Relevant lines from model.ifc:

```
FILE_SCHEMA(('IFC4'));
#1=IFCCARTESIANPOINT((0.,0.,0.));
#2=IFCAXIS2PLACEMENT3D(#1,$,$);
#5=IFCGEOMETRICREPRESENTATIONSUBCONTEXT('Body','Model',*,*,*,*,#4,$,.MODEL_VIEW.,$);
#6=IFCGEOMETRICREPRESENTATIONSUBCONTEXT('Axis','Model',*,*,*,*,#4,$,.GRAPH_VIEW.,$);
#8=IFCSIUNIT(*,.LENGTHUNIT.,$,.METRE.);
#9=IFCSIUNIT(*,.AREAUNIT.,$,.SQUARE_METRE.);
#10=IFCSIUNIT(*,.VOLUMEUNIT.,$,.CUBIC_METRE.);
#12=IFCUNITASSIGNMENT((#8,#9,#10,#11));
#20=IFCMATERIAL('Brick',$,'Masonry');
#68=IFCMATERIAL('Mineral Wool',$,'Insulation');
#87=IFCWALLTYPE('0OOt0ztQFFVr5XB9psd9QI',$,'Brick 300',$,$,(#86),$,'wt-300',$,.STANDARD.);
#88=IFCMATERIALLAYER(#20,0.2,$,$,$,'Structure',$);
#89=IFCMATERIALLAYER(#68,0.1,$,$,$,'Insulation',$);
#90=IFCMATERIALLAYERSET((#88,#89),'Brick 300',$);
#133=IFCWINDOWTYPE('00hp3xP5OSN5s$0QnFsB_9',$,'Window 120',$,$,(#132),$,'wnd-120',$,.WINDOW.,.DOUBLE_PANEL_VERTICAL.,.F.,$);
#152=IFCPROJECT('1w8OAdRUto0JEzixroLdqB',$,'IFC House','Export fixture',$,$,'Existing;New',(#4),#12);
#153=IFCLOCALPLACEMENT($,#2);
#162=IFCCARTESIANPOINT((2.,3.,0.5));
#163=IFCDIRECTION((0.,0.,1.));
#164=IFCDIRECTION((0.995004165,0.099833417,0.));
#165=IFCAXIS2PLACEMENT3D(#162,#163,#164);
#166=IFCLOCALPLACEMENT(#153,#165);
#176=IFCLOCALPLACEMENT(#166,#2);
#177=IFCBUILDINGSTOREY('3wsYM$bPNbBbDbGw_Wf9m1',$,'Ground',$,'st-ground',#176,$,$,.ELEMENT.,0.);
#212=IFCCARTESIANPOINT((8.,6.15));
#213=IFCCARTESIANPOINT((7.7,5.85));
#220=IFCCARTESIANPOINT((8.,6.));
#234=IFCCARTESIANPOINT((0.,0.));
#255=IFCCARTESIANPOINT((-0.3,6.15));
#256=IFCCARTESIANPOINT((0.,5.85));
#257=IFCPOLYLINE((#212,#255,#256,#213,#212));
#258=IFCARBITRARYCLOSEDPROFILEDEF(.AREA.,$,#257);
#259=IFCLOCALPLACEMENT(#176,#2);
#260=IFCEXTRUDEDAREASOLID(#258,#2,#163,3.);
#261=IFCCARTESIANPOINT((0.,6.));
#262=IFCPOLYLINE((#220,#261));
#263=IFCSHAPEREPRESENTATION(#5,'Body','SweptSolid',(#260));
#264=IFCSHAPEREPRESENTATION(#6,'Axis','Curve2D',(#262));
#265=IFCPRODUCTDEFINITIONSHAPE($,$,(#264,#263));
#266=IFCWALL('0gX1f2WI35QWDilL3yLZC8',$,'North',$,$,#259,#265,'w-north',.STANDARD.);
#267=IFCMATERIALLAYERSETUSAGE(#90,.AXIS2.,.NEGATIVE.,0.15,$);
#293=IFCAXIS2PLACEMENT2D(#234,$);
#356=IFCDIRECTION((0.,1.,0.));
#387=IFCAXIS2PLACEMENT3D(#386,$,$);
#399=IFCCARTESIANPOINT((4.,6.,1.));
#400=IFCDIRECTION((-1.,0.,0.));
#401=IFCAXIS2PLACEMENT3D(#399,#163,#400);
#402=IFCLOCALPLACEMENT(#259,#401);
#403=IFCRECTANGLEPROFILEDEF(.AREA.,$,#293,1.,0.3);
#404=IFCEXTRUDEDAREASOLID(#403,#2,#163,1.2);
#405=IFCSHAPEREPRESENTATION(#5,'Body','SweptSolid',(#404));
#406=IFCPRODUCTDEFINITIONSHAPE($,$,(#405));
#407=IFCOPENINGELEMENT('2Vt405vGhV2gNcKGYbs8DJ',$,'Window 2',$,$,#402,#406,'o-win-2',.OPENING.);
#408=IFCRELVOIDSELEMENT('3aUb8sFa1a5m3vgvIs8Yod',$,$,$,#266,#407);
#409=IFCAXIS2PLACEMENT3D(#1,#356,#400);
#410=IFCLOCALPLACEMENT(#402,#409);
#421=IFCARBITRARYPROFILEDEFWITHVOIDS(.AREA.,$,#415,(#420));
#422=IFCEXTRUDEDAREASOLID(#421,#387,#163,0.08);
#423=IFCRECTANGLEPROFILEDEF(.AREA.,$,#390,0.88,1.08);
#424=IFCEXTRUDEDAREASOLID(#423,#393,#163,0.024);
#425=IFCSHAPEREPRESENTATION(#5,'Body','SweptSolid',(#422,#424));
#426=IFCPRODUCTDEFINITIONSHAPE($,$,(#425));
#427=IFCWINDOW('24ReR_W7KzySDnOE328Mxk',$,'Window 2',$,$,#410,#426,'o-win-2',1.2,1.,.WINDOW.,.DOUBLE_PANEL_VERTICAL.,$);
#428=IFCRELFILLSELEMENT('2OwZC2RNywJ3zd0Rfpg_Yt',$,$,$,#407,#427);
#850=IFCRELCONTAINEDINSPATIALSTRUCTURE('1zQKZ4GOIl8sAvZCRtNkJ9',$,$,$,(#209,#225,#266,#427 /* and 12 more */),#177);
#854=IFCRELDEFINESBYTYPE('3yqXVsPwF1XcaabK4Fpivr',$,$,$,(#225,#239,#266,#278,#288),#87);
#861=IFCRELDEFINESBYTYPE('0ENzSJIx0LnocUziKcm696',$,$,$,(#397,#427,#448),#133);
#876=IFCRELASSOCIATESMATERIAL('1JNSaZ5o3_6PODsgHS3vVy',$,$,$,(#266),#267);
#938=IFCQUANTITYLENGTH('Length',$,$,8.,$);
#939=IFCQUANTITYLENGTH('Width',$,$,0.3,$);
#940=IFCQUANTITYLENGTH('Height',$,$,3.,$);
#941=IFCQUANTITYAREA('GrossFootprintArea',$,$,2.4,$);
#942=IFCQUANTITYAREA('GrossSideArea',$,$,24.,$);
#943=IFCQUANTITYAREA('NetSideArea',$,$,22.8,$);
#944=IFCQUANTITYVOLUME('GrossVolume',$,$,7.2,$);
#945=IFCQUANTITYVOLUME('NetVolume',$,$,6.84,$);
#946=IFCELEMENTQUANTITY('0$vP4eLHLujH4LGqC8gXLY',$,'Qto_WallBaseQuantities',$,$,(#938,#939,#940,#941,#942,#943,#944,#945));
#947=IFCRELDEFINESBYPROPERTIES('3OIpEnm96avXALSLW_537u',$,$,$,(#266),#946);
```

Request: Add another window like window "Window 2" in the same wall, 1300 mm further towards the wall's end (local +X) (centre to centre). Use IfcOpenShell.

```python
import ifcopenshell
import ifcopenshell.api.feature
import ifcopenshell.api.geometry
import ifcopenshell.api.pset
import ifcopenshell.api.root
import ifcopenshell.geom
import ifcopenshell.util.element
import ifcopenshell.util.placement
import ifcopenshell.util.shape
import ifcopenshell.util.unit

model = ifcopenshell.open("model.ifc")
unit_scale = ifcopenshell.util.unit.calculate_unit_scale(model)
area_scale = ifcopenshell.util.unit.calculate_unit_scale(model, "AREAUNIT")
volume_scale = ifcopenshell.util.unit.calculate_unit_scale(model, "VOLUMEUNIT")
settings = ifcopenshell.geom.settings()


def volume(element):
    """Net volume in cubic metres, openings subtracted."""
    shape = ifcopenshell.geom.create_shape(settings, element)
    return ifcopenshell.util.shape.get_volume(shape.geometry)


window = model.by_guid("24ReR_W7KzySDnOE328Mxk")
opening = window.FillsVoids[0].RelatingOpeningElement
wall = opening.VoidsElements[0].RelatingBuildingElement
before = volume(wall)
shift = ifcopenshell.util.placement.get_local_placement(wall.ObjectPlacement)[:3, 0] * 1.3 / unit_scale

# copy_class copies the void relationship, type, container and properties, but no geometry.
new_opening = ifcopenshell.api.root.copy_class(model, product=opening)
new_opening.Representation = ifcopenshell.util.element.copy_deep(
    model, opening.Representation, exclude=["IfcGeometricRepresentationContext", "IfcRepresentationMap"]
)
new_opening.Tag = None
new_window = ifcopenshell.api.root.copy_class(model, product=window)
new_window.Representation = ifcopenshell.util.element.copy_deep(
    model, window.Representation, exclude=["IfcGeometricRepresentationContext", "IfcRepresentationMap"]
)
new_window.Tag = None
ifcopenshell.api.feature.add_filling(model, opening=new_opening, element=new_window)

for old, new in ((opening, new_opening), (window, new_window)):
    matrix = ifcopenshell.util.placement.get_local_placement(old.ObjectPlacement)
    matrix[:3, 3] += shift
    ifcopenshell.api.geometry.edit_object_placement(model, product=new, matrix=matrix, is_si=False)

after = volume(wall)
thickness = 0.3  # wall thickness in metres

# Update the wall's stored quantities.
qto = model.by_id(ifcopenshell.util.element.get_pset(wall, "Qto_WallBaseQuantities", should_inherit=False)["id"])
ifcopenshell.api.pset.edit_qto(model, qto=qto, properties={
    "NetSideArea": after / thickness / area_scale,
    "NetVolume": after / volume_scale,
})

print(f"wall volume {before:.3f} -> {after:.3f} m3")

model.write("model_updated.ifc")
```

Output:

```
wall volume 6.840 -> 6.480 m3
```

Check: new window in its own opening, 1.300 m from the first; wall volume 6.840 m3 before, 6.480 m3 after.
